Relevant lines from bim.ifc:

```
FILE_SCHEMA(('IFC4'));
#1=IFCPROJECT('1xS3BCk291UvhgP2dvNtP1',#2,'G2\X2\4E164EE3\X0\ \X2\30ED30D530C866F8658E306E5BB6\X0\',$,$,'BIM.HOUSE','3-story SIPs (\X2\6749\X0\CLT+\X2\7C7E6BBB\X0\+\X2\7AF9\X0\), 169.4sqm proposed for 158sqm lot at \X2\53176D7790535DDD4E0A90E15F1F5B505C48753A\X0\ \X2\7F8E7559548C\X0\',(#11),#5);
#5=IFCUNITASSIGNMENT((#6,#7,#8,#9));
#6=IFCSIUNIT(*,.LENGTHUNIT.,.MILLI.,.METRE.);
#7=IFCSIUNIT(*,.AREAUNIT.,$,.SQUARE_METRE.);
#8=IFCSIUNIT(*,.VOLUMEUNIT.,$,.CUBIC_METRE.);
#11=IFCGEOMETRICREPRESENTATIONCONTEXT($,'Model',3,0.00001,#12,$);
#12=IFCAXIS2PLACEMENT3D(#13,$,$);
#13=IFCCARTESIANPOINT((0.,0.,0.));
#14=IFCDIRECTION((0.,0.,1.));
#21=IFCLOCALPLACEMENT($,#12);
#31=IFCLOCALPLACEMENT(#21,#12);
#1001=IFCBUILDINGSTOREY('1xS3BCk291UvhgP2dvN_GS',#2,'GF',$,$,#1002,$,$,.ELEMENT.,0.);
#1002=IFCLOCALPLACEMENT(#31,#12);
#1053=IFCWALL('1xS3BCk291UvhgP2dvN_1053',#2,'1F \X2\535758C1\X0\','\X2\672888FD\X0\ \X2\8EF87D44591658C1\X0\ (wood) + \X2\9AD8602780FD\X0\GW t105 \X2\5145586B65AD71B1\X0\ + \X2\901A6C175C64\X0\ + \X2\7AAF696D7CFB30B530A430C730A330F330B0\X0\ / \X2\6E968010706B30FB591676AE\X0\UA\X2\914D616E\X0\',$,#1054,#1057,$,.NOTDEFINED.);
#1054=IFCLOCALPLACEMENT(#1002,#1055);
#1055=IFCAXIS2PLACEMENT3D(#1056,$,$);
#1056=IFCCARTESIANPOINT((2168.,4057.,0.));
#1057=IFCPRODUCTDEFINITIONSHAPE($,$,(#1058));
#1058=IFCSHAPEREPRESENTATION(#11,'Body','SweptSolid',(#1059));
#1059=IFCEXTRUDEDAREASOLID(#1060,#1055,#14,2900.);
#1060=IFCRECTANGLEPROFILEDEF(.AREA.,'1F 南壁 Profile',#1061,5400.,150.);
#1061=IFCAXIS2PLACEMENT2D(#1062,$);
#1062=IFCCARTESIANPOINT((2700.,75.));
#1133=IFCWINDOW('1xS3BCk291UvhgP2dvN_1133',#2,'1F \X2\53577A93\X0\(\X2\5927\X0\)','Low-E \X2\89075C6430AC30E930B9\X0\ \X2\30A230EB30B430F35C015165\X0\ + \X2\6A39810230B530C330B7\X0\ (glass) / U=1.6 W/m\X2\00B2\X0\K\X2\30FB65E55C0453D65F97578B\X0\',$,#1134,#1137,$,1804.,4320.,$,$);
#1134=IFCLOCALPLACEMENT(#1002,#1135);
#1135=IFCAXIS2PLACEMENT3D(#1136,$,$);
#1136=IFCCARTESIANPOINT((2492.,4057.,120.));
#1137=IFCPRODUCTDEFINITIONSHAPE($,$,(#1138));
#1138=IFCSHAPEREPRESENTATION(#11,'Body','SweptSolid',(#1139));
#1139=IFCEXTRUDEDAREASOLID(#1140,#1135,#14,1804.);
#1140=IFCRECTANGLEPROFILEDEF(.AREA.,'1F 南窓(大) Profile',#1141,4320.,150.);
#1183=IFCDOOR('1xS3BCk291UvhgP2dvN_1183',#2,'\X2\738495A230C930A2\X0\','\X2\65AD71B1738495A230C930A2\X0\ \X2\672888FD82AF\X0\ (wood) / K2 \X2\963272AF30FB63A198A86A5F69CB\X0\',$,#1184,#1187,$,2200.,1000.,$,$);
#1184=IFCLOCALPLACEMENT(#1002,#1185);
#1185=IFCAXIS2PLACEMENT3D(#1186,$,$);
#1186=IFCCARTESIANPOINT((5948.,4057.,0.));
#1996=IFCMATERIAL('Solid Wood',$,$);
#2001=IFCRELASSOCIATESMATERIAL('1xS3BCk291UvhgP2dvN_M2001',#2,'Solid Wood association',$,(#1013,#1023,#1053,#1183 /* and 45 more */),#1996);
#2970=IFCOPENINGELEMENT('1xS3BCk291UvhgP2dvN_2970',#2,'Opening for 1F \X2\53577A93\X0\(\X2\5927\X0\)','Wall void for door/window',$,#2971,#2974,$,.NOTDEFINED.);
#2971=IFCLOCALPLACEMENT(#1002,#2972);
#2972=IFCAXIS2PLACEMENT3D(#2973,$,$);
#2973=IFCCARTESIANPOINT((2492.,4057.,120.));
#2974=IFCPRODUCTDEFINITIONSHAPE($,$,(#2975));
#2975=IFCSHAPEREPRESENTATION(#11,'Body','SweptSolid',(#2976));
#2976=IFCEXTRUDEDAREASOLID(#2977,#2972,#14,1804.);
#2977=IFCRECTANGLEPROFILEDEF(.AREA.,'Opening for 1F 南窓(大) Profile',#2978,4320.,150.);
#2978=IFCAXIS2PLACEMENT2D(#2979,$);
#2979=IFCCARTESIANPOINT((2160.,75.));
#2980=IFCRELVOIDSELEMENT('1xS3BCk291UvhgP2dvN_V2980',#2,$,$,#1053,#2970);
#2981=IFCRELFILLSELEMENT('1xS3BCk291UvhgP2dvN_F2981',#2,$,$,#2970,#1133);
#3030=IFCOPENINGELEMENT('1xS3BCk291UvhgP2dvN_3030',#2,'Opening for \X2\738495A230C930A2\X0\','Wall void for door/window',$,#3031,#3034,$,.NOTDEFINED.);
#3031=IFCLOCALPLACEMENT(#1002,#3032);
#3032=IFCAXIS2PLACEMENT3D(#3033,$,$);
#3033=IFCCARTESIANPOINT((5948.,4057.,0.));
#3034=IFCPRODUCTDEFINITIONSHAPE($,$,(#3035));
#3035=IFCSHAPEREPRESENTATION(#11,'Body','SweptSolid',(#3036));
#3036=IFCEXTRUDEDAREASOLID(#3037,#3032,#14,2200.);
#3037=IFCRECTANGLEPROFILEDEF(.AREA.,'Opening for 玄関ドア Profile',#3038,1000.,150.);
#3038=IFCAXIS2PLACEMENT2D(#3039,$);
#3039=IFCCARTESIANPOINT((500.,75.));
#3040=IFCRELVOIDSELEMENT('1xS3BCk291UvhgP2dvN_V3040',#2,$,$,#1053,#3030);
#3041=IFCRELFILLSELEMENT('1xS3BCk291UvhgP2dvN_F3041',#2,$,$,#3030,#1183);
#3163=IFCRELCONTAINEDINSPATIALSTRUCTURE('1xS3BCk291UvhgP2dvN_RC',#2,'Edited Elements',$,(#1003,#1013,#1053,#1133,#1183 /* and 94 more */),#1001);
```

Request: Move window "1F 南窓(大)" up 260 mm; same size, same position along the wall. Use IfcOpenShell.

```python
import numpy as np
import ifcopenshell
import ifcopenshell.api.geometry
import ifcopenshell.util.placement
import ifcopenshell.util.unit

model = ifcopenshell.open("bim.ifc")
unit_scale = ifcopenshell.util.unit.calculate_unit_scale(model)

window = model.by_guid("1xS3BCk291UvhgP2dvN_1133")
opening = window.FillsVoids[0].RelatingOpeningElement
dz = 260.0

shift = np.array([0.0, 0.0, dz])
# The window is not placed relative to its opening, so move both.
for product in (opening, window):
    matrix = ifcopenshell.util.placement.get_local_placement(product.ObjectPlacement)
    matrix[:3, 3] += shift
    ifcopenshell.api.geometry.edit_object_placement(model, product=product, matrix=matrix, is_si=False)

print(f"moved by {dz * unit_scale:+.3f} m")

model.write("bim_updated.ifc")
```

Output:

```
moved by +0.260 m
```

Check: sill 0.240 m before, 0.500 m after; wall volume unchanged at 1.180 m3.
